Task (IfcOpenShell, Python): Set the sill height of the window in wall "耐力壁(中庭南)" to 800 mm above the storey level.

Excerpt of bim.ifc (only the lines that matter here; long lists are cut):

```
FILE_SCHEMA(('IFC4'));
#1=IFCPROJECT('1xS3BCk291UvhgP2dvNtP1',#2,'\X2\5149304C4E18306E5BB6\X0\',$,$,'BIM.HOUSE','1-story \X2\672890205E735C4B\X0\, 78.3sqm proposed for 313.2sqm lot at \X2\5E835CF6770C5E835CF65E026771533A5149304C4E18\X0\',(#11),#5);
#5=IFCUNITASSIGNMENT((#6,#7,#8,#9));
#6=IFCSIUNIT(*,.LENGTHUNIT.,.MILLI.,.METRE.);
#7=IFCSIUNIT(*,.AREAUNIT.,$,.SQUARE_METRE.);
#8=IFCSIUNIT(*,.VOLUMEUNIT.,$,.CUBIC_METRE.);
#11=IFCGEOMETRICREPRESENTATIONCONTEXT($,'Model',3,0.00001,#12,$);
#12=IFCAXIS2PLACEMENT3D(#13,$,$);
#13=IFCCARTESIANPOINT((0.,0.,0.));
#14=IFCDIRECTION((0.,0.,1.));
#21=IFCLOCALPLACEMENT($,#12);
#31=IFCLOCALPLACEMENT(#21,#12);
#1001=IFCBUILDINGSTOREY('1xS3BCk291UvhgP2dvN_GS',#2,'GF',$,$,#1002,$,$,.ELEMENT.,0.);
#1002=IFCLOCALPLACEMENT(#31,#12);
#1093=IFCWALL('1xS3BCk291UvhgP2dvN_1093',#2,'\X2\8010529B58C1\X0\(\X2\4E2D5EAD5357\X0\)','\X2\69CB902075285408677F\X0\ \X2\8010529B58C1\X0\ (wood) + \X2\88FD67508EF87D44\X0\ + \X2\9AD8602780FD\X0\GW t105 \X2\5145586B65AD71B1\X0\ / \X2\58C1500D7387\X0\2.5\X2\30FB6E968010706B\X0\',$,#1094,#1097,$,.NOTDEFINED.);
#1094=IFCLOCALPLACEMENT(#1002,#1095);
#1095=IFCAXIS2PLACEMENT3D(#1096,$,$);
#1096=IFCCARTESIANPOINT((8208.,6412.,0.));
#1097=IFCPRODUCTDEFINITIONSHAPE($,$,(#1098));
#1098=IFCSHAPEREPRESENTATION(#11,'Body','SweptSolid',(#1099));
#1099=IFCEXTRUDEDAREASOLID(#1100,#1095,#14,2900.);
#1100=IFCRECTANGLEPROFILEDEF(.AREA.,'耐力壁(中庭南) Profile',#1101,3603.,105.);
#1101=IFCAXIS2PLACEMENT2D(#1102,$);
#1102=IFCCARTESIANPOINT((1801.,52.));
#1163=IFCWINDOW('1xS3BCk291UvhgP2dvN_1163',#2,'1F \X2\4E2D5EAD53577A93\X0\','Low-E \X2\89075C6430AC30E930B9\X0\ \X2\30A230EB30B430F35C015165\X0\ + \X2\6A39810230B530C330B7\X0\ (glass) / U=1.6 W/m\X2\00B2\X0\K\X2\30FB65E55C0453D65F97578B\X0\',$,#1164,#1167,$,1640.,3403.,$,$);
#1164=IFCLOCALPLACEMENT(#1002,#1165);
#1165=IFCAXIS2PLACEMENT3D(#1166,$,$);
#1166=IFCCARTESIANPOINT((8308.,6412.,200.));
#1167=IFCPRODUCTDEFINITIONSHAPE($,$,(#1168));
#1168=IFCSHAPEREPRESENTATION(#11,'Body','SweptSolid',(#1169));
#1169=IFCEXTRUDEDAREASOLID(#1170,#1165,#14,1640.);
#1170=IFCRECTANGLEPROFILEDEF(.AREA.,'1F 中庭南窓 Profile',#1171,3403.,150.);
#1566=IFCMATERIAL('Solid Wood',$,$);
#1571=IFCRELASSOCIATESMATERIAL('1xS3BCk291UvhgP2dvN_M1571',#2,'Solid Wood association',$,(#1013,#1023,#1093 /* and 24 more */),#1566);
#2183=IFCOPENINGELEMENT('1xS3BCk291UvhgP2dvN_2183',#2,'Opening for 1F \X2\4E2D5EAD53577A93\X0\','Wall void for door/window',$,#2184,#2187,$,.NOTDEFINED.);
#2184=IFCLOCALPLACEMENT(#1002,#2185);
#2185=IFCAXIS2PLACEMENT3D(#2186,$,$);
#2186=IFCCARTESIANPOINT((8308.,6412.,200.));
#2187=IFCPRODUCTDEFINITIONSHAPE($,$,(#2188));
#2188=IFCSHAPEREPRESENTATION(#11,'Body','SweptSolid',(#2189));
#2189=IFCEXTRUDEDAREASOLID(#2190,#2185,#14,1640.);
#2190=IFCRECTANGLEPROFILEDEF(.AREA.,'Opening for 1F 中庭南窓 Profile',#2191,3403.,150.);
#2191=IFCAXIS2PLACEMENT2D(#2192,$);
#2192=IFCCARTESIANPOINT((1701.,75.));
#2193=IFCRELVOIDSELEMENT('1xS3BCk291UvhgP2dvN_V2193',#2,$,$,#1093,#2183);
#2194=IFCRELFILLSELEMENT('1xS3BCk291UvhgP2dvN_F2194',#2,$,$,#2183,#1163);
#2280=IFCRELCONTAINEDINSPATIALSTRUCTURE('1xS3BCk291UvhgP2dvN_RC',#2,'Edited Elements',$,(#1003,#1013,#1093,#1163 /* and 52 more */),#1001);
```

```python
import numpy as np
import ifcopenshell
import ifcopenshell.api.geometry
import ifcopenshell.geom
import ifcopenshell.util.element
import ifcopenshell.util.placement
import ifcopenshell.util.shape
import ifcopenshell.util.unit

model = ifcopenshell.open("bim.ifc")
unit_scale = ifcopenshell.util.unit.calculate_unit_scale(model)

window = model.by_guid("1xS3BCk291UvhgP2dvN_1163")
opening = window.FillsVoids[0].RelatingOpeningElement
storey = ifcopenshell.util.element.get_container(window, ifc_class="IfcBuildingStorey")
level = ifcopenshell.util.placement.get_local_placement(storey.ObjectPlacement)[2, 3]

# The opening's origin need not be at the sill, so measure its lowest point.
shape = ifcopenshell.geom.create_shape(ifcopenshell.geom.settings(), opening)
bottom = ifcopenshell.util.shape.get_shape_bottom_elevation(shape, shape.geometry) / unit_scale
dz = level + 800.0 - bottom

shift = np.array([0.0, 0.0, dz])
# The window is not placed relative to its opening, so move both.
for product in (opening, window):
    matrix = ifcopenshell.util.placement.get_local_placement(product.ObjectPlacement)
    matrix[:3, 3] += shift
    ifcopenshell.api.geometry.edit_object_placement(model, product=product, matrix=matrix, is_si=False)

print(f"moved by {dz * unit_scale:+.3f} m")

model.write("bim_edited.ifc")
```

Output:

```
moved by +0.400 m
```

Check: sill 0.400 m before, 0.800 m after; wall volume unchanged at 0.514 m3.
